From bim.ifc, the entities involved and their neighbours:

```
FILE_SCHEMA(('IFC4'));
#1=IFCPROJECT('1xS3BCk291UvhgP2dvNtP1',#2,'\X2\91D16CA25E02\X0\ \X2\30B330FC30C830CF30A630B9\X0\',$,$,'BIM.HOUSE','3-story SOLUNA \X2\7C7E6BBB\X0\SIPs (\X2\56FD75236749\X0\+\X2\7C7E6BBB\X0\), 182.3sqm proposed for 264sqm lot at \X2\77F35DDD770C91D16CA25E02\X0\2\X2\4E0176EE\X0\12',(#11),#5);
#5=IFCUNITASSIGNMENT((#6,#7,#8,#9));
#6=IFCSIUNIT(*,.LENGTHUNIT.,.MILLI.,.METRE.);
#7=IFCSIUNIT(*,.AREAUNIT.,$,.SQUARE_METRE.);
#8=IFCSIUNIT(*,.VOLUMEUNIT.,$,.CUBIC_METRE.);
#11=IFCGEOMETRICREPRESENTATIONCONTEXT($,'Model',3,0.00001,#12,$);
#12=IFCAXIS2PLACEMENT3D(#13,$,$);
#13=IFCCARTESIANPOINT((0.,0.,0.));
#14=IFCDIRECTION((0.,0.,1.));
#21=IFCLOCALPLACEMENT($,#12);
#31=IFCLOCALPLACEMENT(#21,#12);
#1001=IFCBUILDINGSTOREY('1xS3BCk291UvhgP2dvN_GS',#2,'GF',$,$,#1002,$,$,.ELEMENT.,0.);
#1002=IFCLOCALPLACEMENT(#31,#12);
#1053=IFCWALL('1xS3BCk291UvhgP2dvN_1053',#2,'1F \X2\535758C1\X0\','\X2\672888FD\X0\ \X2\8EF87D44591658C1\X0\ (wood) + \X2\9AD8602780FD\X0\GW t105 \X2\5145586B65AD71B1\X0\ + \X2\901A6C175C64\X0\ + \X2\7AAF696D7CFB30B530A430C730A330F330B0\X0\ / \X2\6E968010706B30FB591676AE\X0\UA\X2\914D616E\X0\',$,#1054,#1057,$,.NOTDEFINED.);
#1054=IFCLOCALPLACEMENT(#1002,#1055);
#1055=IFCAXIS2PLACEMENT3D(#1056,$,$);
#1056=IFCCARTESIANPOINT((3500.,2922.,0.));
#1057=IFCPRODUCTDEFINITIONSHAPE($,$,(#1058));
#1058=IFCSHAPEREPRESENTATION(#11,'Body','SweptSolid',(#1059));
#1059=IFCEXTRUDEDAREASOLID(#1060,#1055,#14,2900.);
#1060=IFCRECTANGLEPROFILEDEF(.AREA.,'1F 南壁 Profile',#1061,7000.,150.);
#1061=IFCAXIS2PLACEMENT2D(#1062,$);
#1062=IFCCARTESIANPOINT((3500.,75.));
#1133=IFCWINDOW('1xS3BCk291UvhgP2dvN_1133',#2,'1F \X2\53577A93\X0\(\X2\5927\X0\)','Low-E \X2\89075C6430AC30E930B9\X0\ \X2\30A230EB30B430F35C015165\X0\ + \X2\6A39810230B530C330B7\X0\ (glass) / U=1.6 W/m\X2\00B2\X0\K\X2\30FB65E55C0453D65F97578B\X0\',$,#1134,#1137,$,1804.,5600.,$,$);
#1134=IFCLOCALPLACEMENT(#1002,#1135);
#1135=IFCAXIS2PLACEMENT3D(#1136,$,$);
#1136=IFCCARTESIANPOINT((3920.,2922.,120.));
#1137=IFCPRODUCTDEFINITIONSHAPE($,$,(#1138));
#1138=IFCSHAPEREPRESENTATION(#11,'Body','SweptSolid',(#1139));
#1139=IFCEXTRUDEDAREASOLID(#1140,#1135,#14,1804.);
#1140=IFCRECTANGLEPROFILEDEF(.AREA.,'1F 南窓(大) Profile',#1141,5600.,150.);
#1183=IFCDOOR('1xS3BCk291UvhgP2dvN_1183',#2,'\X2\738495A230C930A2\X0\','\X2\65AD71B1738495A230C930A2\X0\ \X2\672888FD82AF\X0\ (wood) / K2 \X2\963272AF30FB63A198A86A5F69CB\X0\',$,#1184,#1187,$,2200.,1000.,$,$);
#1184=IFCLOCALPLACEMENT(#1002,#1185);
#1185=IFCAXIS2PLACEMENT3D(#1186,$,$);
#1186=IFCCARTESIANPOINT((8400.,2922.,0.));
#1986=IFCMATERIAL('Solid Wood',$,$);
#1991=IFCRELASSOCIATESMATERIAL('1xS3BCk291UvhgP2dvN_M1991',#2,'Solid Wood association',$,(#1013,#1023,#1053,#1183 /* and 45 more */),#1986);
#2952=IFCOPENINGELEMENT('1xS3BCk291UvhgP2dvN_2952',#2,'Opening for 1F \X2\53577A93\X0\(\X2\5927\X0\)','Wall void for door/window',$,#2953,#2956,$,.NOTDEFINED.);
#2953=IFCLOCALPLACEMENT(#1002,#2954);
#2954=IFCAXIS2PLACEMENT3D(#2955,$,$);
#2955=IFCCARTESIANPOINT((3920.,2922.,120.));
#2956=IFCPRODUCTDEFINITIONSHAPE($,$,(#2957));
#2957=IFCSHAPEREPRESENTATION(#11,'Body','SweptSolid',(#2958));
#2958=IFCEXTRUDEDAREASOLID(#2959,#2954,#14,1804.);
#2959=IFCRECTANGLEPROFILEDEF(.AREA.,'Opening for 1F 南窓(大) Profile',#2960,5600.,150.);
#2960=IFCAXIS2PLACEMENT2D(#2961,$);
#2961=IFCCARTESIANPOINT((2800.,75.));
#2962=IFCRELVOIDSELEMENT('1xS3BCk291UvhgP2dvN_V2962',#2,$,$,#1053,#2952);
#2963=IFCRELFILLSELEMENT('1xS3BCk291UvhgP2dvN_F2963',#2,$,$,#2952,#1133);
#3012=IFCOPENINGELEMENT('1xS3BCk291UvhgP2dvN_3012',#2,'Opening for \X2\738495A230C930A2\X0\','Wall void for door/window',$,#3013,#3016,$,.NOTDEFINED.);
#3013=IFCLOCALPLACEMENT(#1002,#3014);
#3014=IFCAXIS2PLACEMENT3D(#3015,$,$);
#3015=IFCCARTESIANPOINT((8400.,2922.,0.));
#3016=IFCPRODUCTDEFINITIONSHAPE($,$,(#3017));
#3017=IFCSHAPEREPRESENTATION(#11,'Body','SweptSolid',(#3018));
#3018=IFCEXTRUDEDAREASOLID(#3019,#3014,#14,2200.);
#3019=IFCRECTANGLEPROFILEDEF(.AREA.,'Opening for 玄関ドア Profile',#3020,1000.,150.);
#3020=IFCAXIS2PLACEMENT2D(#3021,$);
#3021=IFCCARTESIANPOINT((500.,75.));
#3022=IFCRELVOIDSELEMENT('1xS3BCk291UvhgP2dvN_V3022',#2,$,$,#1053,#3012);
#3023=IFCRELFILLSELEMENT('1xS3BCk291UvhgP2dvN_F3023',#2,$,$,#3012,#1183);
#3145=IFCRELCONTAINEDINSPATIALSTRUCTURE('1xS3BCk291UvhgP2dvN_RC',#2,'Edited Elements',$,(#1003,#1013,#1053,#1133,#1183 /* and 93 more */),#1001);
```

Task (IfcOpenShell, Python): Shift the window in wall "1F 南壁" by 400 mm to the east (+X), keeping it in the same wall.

```python
import ifcopenshell
import ifcopenshell.api.geometry
import ifcopenshell.util.placement

model = ifcopenshell.open("bim.ifc")

window = model.by_guid("1xS3BCk291UvhgP2dvN_1133")
opening = window.FillsVoids[0].RelatingOpeningElement
wall = opening.VoidsElements[0].RelatingBuildingElement

wall_matrix = ifcopenshell.util.placement.get_local_placement(wall.ObjectPlacement)
shift = wall_matrix[:3, 0] * 400.0
before = ifcopenshell.util.placement.get_local_placement(window.ObjectPlacement)[:3, 3].copy()

# The window is not placed relative to its opening, so move both.
for product in (opening, window):
    matrix = ifcopenshell.util.placement.get_local_placement(product.ObjectPlacement)
    matrix[:3, 3] += shift
    ifcopenshell.api.geometry.edit_object_placement(model, product=product, matrix=matrix, is_si=False)

after = ifcopenshell.util.placement.get_local_placement(window.ObjectPlacement)[:3, 3]
print("window moved by", (after - before).round(3) + 0.0)

model.write("bim_edited.ifc")
```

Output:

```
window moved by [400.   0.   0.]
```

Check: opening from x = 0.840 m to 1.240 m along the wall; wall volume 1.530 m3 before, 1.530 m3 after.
